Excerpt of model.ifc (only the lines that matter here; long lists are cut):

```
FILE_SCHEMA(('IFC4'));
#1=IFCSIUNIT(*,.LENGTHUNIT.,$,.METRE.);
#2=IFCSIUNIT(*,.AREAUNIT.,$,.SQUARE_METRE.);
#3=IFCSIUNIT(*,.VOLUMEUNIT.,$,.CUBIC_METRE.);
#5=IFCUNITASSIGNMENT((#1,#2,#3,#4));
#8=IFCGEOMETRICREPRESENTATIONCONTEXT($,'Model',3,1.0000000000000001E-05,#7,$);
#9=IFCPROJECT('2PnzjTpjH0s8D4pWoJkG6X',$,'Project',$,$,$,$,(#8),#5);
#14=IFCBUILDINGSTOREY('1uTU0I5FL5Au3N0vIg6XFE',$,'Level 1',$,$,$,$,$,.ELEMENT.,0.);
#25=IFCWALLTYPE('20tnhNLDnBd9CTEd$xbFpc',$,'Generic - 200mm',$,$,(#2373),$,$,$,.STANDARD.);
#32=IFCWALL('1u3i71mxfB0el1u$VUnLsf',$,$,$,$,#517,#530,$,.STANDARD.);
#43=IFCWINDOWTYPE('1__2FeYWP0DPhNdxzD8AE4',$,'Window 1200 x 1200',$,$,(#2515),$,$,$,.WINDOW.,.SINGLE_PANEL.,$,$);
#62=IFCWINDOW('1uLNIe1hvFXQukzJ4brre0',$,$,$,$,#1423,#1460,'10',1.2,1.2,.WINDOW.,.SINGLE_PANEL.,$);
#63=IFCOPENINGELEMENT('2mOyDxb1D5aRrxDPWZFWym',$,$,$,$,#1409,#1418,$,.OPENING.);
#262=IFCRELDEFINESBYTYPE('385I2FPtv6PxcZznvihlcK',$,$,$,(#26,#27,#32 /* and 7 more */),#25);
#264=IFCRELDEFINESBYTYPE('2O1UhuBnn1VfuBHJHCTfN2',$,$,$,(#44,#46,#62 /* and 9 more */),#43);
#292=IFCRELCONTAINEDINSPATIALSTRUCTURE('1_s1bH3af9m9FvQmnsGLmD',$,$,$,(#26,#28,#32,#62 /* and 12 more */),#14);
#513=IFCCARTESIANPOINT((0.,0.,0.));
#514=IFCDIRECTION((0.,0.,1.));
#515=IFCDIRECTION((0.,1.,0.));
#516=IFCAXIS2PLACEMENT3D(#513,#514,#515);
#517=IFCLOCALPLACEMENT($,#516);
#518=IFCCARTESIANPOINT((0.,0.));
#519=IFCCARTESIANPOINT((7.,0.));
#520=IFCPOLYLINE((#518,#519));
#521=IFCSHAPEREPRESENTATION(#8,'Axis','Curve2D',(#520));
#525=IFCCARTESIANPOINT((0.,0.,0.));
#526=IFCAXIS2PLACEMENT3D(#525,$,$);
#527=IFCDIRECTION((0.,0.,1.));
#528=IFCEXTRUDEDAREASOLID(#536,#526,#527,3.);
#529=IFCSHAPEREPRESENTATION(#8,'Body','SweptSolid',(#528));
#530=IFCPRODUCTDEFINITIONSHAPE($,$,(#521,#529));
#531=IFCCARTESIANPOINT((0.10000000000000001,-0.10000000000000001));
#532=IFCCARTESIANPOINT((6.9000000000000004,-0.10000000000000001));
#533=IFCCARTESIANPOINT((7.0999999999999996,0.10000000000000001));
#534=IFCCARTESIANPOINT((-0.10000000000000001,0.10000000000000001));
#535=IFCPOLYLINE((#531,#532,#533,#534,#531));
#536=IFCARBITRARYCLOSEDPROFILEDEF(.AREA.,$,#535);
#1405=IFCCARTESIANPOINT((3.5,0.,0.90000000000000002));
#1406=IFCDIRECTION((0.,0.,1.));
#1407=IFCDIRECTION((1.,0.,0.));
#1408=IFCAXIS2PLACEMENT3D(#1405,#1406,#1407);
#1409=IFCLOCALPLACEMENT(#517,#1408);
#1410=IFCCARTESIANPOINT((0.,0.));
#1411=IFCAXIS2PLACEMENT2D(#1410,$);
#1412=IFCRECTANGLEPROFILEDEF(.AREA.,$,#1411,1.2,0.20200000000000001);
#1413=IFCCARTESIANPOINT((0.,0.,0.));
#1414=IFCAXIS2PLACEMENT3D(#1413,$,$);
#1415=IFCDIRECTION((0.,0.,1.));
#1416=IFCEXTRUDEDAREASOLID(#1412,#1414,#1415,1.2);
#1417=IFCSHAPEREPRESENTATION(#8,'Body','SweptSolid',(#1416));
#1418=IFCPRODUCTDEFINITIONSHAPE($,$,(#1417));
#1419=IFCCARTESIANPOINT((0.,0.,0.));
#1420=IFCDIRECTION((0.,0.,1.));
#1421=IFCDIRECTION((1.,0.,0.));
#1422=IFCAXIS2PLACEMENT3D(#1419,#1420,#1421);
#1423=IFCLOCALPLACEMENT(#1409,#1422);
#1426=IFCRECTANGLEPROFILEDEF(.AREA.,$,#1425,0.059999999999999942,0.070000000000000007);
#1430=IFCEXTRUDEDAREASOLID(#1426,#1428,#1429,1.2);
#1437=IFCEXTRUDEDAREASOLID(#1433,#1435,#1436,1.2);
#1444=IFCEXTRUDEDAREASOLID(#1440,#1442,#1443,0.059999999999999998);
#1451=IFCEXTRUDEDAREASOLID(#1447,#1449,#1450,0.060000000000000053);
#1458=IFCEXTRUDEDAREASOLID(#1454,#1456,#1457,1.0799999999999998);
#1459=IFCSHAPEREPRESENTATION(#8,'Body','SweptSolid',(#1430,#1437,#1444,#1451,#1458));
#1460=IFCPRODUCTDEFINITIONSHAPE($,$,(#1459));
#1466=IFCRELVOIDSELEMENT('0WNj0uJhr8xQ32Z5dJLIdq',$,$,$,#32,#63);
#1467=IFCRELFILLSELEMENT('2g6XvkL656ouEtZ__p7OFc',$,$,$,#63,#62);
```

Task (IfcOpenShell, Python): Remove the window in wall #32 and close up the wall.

```python
import ifcopenshell
import ifcopenshell.api.feature
import ifcopenshell.api.root
import ifcopenshell.geom
import ifcopenshell.util.shape

model = ifcopenshell.open("model.ifc")
settings = ifcopenshell.geom.settings()


def volume(element):
    """Net volume in cubic metres, openings subtracted."""
    shape = ifcopenshell.geom.create_shape(settings, element)
    return ifcopenshell.util.shape.get_volume(shape.geometry)


window = model.by_guid("1uLNIe1hvFXQukzJ4brre0")
opening = window.FillsVoids[0].RelatingOpeningElement
wall = opening.VoidsElements[0].RelatingBuildingElement
before = volume(wall)

ifcopenshell.api.root.remove_product(model, product=window)
ifcopenshell.api.feature.remove_feature(model, feature=opening)

after = volume(wall)

print(f"wall volume {before:.3f} -> {after:.3f} m3")

model.write("model_edited.ifc")
```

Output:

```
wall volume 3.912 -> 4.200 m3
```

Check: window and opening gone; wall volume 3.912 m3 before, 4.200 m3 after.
